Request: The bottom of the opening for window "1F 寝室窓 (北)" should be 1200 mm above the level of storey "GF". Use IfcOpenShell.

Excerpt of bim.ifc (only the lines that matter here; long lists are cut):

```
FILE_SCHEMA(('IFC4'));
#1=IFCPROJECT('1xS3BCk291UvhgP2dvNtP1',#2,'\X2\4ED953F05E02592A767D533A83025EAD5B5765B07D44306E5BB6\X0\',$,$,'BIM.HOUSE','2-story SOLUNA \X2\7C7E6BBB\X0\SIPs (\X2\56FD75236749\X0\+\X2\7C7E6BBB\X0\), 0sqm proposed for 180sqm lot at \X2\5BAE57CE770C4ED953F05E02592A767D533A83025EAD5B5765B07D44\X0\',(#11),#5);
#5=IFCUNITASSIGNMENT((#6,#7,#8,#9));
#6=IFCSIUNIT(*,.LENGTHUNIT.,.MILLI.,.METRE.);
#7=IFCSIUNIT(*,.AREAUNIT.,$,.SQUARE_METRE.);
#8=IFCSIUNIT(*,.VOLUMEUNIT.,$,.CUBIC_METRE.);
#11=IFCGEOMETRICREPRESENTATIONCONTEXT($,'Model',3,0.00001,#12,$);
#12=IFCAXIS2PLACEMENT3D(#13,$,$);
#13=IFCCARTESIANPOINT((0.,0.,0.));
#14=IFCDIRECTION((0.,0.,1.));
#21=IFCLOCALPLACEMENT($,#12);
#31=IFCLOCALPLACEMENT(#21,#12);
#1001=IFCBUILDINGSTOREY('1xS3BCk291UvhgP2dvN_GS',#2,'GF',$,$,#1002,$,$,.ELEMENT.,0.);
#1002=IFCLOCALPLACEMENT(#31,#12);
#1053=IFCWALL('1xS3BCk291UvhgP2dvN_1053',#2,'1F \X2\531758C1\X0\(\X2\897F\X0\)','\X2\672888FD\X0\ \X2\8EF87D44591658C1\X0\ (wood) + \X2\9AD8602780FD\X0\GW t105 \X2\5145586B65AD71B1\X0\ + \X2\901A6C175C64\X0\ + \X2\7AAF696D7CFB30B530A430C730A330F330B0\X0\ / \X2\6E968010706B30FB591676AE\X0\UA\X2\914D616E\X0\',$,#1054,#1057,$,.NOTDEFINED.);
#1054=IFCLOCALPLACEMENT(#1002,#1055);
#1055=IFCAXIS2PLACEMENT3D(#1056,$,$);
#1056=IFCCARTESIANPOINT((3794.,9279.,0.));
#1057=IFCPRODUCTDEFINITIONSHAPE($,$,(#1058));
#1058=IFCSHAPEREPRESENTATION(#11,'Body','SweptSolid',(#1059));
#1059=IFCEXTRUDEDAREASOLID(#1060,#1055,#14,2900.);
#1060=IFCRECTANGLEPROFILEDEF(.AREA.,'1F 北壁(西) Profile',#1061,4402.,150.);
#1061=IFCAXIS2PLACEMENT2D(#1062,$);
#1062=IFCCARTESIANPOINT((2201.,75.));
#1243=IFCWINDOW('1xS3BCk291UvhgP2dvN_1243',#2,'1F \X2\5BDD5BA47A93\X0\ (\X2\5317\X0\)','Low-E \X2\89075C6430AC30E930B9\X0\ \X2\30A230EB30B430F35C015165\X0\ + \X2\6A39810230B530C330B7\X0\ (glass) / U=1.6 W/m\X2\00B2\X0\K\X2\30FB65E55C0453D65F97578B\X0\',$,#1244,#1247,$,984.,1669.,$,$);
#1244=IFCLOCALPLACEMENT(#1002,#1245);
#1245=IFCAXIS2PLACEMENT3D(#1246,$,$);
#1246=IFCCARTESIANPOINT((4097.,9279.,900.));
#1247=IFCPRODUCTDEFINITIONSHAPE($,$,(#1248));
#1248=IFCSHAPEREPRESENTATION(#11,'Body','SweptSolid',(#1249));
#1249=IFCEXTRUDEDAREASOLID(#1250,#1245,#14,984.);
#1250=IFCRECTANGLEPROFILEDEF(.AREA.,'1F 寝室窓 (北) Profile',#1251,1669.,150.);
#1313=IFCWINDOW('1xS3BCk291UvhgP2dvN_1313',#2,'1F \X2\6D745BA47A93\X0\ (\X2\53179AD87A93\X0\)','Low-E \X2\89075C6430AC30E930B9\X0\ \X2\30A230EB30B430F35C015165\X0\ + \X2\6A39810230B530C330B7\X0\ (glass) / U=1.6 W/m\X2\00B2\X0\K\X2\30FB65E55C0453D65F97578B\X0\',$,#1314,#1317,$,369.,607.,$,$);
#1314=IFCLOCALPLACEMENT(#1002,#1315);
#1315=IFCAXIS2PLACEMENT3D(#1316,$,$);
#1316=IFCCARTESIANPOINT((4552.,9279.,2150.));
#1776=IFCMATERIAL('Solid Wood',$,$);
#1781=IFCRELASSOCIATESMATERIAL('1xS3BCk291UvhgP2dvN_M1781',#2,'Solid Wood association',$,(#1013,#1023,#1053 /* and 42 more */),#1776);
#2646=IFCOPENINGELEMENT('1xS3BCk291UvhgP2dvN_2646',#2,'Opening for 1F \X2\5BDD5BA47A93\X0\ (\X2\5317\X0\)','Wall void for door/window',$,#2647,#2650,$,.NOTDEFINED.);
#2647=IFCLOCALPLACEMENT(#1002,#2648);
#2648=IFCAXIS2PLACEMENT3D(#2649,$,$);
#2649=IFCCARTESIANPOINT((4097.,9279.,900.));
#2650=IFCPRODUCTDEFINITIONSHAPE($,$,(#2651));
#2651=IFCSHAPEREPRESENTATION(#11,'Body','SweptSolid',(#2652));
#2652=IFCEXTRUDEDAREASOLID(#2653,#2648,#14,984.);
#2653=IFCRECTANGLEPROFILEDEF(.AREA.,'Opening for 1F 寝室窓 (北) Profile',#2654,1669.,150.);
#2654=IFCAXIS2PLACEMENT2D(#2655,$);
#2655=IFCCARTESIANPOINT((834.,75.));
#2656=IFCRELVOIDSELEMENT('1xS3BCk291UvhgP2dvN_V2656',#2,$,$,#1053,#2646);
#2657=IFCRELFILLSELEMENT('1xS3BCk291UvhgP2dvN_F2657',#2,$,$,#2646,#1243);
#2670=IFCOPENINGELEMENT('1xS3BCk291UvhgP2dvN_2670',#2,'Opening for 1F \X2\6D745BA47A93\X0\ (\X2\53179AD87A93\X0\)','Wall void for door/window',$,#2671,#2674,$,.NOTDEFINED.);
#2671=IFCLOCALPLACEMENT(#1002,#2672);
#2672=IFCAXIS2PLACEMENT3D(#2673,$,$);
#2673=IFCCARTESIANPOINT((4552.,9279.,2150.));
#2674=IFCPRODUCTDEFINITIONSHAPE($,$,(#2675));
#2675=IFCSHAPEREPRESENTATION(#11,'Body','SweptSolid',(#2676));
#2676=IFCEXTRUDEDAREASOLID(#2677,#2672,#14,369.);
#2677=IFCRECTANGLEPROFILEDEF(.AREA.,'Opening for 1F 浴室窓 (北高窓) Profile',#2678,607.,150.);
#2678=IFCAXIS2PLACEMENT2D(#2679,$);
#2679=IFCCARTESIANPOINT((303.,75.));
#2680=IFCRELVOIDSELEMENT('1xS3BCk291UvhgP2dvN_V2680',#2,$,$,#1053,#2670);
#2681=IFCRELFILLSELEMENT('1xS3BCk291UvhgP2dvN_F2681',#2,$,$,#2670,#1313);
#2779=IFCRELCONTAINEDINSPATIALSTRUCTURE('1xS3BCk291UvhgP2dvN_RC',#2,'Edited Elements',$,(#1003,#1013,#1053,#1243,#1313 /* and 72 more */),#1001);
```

```python
import numpy as np
import ifcopenshell
import ifcopenshell.api.geometry
import ifcopenshell.geom
import ifcopenshell.util.element
import ifcopenshell.util.placement
import ifcopenshell.util.shape
import ifcopenshell.util.unit

model = ifcopenshell.open("bim.ifc")
unit_scale = ifcopenshell.util.unit.calculate_unit_scale(model)

window = model.by_guid("1xS3BCk291UvhgP2dvN_1243")
opening = window.FillsVoids[0].RelatingOpeningElement
storey = ifcopenshell.util.element.get_container(window, ifc_class="IfcBuildingStorey")
level = ifcopenshell.util.placement.get_local_placement(storey.ObjectPlacement)[2, 3]

# The opening's origin need not be at the sill, so measure its lowest point.
shape = ifcopenshell.geom.create_shape(ifcopenshell.geom.settings(), opening)
bottom = ifcopenshell.util.shape.get_shape_bottom_elevation(shape, shape.geometry) / unit_scale
dz = level + 1.2 / unit_scale - bottom

shift = np.array([0.0, 0.0, dz])
# The window is not placed relative to its opening, so move both.
for product in (opening, window):
    matrix = ifcopenshell.util.placement.get_local_placement(product.ObjectPlacement)
    matrix[:3, 3] += shift
    ifcopenshell.api.geometry.edit_object_placement(model, product=product, matrix=matrix, is_si=False)

print(f"moved by {dz * unit_scale:+.3f} m")

model.write("bim_v2.ifc")
```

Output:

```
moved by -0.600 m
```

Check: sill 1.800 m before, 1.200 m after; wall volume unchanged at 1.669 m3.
